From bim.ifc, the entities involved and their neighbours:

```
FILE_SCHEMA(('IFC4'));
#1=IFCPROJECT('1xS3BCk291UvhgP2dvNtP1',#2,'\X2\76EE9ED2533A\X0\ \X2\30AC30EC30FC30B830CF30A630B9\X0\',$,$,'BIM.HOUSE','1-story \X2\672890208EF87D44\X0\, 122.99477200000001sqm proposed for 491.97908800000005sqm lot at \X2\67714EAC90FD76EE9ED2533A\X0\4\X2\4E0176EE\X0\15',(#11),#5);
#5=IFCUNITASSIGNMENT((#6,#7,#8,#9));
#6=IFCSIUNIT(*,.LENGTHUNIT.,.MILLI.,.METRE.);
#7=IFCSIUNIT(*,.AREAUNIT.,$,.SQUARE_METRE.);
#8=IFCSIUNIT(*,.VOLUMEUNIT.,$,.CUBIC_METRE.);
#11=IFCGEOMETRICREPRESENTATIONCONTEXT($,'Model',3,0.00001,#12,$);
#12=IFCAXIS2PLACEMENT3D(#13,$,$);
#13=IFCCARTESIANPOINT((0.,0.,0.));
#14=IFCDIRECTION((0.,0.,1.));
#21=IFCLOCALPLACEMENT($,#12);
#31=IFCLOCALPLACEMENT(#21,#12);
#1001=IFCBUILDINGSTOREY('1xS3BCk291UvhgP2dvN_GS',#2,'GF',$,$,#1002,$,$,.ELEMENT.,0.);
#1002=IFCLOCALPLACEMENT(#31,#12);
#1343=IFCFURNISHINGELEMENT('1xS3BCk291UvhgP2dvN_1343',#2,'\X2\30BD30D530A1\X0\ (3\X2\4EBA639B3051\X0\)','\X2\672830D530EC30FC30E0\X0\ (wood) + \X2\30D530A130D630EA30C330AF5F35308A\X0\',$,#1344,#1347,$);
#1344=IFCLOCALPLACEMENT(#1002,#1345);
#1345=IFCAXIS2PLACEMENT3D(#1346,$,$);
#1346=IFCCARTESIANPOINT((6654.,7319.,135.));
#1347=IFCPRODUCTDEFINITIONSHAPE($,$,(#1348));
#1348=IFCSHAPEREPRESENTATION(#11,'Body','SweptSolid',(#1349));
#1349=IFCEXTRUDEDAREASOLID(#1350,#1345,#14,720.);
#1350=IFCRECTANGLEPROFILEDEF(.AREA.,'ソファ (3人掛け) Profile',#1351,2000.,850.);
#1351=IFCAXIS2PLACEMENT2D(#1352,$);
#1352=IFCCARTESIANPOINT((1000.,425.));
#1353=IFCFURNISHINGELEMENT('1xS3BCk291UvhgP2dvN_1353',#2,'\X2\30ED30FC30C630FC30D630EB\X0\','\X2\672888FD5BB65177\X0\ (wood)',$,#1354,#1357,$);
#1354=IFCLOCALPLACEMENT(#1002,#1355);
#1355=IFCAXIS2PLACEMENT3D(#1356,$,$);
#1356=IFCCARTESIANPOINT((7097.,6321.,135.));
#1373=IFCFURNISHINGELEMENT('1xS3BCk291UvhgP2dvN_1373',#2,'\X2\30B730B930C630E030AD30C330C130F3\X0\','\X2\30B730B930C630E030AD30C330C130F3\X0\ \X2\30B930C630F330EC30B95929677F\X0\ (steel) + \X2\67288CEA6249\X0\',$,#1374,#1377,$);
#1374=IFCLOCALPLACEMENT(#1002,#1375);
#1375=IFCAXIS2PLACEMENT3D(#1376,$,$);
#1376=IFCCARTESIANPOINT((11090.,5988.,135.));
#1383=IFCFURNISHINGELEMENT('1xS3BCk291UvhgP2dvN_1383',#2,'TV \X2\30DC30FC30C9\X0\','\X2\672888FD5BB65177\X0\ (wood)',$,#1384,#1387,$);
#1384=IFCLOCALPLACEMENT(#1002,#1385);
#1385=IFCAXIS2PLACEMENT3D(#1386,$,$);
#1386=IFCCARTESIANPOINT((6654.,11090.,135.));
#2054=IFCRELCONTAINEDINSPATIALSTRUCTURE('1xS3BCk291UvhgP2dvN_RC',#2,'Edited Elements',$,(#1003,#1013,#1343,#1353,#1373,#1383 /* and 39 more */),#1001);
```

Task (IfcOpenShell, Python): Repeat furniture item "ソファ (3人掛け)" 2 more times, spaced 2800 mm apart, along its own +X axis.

```python
import ifcopenshell
import ifcopenshell.api.geometry
import ifcopenshell.api.root
import ifcopenshell.util.element
import ifcopenshell.util.placement
import ifcopenshell.util.unit

model = ifcopenshell.open("bim.ifc")
unit_scale = ifcopenshell.util.unit.calculate_unit_scale(model)


def reuse_history(source, copy):
    """copy_class also copies each property set's owner history, people and application; keep the originals."""
    for rel in copy.IsDefinedBy:
        if rel.is_a("IfcRelDefinesByProperties") and (history := rel.RelatingPropertyDefinition.OwnerHistory):
            rel.RelatingPropertyDefinition.OwnerHistory = source.OwnerHistory
            ifcopenshell.util.element.remove_deep2(model, history)


source = model.by_guid("1xS3BCk291UvhgP2dvN_1343")
base = ifcopenshell.util.placement.get_local_placement(source.ObjectPlacement)
step = base[:3, 0] * 2.8 / unit_scale

for i in range(1, 3):
    copy = ifcopenshell.api.root.copy_class(model, product=source)
    copy.Representation = ifcopenshell.util.element.copy_deep(
        model, source.Representation, exclude=["IfcGeometricRepresentationContext", "IfcRepresentationMap"]
    )
    reuse_history(source, copy)
    matrix = base.copy()
    matrix[:3, 3] += i * step
    print("added at", matrix[:3, 3].round(3) + 0.0)
    ifcopenshell.api.geometry.edit_object_placement(model, product=copy, matrix=matrix, is_si=False)

model.write("bim_updated.ifc")
```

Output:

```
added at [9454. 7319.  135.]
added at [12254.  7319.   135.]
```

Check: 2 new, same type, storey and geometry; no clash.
